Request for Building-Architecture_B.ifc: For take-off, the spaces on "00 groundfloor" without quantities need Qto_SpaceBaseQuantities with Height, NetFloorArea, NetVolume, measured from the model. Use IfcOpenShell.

First a look at what the model holds.

```python
import ifcopenshell
import ifcopenshell.util.element
import ifcopenshell.util.unit

model = ifcopenshell.open("Building-Architecture_B.ifc")
print(model.schema)
for unit_type in ("LENGTHUNIT", "AREAUNIT", "VOLUMEUNIT"):
    print(unit_type, ifcopenshell.util.unit.calculate_unit_scale(model, unit_type))
storey = next(s for s in model.by_type("IfcBuildingStorey") if s.Name == "00 groundfloor")
spaces = [e for e in ifcopenshell.util.element.get_decomposition(storey) if e.is_a("IfcSpace")]
for e in sorted(spaces, key=lambda e: e.id()):
    print(e.id(), e.is_a(), e.Name, list(ifcopenshell.util.element.get_psets(e, qtos_only=True)), sep=" | ")
```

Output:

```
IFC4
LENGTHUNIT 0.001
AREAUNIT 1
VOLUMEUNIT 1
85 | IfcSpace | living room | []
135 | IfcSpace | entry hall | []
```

```python
import ifcopenshell
import ifcopenshell.api.pset
import ifcopenshell.geom
import ifcopenshell.util.element
import ifcopenshell.util.shape
import ifcopenshell.util.unit

model = ifcopenshell.open("Building-Architecture_B.ifc")
unit_scale = ifcopenshell.util.unit.calculate_unit_scale(model)
area_scale = ifcopenshell.util.unit.calculate_unit_scale(model, "AREAUNIT")
volume_scale = ifcopenshell.util.unit.calculate_unit_scale(model, "VOLUMEUNIT")
settings = ifcopenshell.geom.settings()

storey = next(s for s in model.by_type("IfcBuildingStorey") if s.Name == "00 groundfloor")
spaces = [e for e in ifcopenshell.util.element.get_decomposition(storey) if e.is_a("IfcSpace")]

for e in sorted(spaces, key=lambda e: e.id()):
    if ifcopenshell.util.element.get_psets(e, qtos_only=True, should_inherit=False):
        continue
    # Geometry comes back in metres, in the element's own axes.
    shape = ifcopenshell.geom.create_shape(settings, e)
    values = {
        "Height": ifcopenshell.util.shape.get_z(shape.geometry) / unit_scale,
        "NetFloorArea": ifcopenshell.util.shape.get_footprint_area(shape.geometry) / area_scale,
        "NetVolume": ifcopenshell.util.shape.get_volume(shape.geometry) / volume_scale,
    }
    qto = ifcopenshell.api.pset.add_qto(model, product=e, name="Qto_SpaceBaseQuantities")
    ifcopenshell.api.pset.edit_qto(model, qto=qto, properties=values)
    print(e.id(), {k: round(v, 3) for k, v in values.items()})

model.write("Building-Architecture_B-out.ifc")
```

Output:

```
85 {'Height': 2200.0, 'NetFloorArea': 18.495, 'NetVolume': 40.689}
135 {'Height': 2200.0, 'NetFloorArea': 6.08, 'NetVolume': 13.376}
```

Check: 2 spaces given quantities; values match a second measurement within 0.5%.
